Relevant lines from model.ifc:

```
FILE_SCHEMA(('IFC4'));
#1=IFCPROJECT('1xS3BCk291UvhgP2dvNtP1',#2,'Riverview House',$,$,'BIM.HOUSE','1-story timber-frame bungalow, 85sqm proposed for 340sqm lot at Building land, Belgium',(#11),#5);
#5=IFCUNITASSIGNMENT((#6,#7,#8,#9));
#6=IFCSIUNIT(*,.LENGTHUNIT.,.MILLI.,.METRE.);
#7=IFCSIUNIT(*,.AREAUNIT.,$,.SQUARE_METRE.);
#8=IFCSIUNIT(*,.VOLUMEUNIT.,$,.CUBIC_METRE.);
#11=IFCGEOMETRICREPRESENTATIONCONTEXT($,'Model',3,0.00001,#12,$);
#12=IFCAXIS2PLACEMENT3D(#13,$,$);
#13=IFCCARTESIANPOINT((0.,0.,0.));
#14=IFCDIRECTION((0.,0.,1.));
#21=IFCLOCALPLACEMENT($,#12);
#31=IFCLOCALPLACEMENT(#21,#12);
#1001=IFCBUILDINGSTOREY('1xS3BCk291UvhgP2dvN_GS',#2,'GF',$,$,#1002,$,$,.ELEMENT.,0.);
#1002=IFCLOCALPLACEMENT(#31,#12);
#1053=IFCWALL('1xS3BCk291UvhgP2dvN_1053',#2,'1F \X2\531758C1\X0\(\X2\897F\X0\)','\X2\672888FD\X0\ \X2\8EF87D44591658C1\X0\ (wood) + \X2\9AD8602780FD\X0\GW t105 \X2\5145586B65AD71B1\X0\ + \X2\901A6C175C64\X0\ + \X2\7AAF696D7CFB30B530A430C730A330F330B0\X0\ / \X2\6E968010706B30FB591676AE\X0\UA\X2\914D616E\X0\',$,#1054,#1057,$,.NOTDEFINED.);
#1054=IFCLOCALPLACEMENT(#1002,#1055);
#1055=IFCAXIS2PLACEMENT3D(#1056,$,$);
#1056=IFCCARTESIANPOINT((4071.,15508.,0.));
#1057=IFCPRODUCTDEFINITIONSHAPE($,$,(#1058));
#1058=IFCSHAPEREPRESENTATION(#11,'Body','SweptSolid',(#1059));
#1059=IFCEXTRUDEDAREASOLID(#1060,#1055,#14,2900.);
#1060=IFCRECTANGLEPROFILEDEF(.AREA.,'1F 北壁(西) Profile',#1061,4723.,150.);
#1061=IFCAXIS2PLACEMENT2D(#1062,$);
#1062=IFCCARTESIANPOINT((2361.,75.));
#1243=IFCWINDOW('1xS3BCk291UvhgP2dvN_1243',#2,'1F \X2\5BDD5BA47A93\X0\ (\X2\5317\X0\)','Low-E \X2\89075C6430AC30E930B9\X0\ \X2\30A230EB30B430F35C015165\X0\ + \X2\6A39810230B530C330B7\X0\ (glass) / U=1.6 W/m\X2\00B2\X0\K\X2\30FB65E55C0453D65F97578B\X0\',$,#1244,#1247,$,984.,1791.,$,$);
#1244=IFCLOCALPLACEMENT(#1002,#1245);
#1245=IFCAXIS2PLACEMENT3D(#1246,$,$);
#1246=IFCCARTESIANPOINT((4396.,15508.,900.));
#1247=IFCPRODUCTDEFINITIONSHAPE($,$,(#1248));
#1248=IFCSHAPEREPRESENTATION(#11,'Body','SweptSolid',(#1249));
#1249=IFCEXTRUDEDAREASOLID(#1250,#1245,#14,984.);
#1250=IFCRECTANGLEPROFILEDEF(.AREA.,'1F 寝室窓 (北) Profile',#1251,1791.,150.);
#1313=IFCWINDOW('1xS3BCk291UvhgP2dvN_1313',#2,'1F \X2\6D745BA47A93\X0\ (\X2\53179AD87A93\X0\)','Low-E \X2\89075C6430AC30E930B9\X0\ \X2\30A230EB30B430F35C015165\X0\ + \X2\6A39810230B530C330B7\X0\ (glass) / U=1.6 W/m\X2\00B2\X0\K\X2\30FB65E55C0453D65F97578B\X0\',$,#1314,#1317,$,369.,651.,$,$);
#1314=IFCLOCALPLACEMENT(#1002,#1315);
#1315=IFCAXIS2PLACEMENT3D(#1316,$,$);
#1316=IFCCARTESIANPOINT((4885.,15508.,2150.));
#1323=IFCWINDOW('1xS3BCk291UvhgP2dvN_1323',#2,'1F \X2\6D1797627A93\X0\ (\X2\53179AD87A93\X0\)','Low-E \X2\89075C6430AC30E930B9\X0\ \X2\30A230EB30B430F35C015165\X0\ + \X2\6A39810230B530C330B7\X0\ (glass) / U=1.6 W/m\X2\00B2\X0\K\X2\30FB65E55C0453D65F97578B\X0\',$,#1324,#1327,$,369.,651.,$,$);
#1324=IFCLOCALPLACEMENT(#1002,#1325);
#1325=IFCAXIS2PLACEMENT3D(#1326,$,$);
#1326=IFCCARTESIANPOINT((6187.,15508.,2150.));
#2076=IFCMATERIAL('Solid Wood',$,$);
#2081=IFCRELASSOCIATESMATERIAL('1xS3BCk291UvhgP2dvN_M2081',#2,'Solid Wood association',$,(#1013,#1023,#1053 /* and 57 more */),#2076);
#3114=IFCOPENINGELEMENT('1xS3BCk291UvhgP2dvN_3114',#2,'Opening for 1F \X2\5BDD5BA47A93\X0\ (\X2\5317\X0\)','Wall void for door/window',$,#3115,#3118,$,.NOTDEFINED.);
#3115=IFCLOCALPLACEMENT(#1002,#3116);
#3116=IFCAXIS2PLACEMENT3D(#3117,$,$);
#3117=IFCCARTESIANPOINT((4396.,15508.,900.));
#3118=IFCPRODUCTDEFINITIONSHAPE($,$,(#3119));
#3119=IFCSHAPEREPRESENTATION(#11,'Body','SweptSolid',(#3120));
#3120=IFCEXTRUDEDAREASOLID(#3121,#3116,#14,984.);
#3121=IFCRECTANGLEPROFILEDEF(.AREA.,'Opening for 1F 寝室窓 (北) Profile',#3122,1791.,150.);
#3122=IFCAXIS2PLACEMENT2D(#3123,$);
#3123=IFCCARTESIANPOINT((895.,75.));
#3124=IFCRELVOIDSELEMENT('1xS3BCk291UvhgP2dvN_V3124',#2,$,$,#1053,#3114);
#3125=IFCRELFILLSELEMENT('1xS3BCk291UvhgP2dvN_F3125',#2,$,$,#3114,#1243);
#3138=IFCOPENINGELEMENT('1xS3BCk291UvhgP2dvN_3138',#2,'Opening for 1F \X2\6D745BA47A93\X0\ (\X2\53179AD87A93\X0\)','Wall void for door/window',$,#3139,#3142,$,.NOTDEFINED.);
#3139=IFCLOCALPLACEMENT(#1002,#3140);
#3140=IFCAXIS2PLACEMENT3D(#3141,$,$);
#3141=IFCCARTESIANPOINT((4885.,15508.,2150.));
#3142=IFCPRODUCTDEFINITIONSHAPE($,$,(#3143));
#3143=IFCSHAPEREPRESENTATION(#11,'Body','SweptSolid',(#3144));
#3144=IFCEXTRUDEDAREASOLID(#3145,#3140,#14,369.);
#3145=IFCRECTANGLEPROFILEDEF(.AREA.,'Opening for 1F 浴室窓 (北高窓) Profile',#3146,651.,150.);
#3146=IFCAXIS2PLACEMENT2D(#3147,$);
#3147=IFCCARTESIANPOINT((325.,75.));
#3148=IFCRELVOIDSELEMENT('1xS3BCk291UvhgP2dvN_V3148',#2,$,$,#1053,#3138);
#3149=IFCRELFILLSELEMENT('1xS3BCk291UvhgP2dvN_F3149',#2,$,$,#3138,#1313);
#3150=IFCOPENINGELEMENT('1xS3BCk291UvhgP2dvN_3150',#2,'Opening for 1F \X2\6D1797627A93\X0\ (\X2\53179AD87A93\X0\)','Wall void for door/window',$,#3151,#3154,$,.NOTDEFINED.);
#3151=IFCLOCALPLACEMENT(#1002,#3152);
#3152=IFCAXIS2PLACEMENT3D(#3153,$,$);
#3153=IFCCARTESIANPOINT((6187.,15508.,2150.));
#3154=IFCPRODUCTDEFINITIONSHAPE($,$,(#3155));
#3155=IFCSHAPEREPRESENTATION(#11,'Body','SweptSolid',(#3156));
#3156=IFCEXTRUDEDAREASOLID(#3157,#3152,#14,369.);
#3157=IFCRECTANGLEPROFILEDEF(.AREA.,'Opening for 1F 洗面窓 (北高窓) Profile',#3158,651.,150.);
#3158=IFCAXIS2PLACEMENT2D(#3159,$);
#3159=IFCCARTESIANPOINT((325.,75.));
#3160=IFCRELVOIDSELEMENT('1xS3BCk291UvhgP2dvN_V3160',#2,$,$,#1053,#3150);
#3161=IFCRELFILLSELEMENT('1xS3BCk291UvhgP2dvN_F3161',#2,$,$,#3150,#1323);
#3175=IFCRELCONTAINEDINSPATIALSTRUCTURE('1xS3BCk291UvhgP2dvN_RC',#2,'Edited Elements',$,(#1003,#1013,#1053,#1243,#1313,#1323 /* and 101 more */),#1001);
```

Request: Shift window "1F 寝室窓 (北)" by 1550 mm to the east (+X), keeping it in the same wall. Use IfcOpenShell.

```python
import ifcopenshell
import ifcopenshell.api.geometry
import ifcopenshell.util.placement

model = ifcopenshell.open("model.ifc")

window = model.by_guid("1xS3BCk291UvhgP2dvN_1243")
opening = window.FillsVoids[0].RelatingOpeningElement
wall = opening.VoidsElements[0].RelatingBuildingElement

wall_matrix = ifcopenshell.util.placement.get_local_placement(wall.ObjectPlacement)
shift = wall_matrix[:3, 0] * 1550.0
before = ifcopenshell.util.placement.get_local_placement(window.ObjectPlacement)[:3, 3].copy()

# The window is not placed relative to its opening, so move both.
for product in (opening, window):
    matrix = ifcopenshell.util.placement.get_local_placement(product.ObjectPlacement)
    matrix[:3, 3] += shift
    ifcopenshell.api.geometry.edit_object_placement(model, product=product, matrix=matrix, is_si=False)

after = ifcopenshell.util.placement.get_local_placement(window.ObjectPlacement)[:3, 3]
print("window moved by", (after - before).round(3) + 0.0)

model.write("model_updated.ifc")
```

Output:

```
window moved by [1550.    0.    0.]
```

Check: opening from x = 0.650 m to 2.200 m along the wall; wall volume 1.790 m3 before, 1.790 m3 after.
